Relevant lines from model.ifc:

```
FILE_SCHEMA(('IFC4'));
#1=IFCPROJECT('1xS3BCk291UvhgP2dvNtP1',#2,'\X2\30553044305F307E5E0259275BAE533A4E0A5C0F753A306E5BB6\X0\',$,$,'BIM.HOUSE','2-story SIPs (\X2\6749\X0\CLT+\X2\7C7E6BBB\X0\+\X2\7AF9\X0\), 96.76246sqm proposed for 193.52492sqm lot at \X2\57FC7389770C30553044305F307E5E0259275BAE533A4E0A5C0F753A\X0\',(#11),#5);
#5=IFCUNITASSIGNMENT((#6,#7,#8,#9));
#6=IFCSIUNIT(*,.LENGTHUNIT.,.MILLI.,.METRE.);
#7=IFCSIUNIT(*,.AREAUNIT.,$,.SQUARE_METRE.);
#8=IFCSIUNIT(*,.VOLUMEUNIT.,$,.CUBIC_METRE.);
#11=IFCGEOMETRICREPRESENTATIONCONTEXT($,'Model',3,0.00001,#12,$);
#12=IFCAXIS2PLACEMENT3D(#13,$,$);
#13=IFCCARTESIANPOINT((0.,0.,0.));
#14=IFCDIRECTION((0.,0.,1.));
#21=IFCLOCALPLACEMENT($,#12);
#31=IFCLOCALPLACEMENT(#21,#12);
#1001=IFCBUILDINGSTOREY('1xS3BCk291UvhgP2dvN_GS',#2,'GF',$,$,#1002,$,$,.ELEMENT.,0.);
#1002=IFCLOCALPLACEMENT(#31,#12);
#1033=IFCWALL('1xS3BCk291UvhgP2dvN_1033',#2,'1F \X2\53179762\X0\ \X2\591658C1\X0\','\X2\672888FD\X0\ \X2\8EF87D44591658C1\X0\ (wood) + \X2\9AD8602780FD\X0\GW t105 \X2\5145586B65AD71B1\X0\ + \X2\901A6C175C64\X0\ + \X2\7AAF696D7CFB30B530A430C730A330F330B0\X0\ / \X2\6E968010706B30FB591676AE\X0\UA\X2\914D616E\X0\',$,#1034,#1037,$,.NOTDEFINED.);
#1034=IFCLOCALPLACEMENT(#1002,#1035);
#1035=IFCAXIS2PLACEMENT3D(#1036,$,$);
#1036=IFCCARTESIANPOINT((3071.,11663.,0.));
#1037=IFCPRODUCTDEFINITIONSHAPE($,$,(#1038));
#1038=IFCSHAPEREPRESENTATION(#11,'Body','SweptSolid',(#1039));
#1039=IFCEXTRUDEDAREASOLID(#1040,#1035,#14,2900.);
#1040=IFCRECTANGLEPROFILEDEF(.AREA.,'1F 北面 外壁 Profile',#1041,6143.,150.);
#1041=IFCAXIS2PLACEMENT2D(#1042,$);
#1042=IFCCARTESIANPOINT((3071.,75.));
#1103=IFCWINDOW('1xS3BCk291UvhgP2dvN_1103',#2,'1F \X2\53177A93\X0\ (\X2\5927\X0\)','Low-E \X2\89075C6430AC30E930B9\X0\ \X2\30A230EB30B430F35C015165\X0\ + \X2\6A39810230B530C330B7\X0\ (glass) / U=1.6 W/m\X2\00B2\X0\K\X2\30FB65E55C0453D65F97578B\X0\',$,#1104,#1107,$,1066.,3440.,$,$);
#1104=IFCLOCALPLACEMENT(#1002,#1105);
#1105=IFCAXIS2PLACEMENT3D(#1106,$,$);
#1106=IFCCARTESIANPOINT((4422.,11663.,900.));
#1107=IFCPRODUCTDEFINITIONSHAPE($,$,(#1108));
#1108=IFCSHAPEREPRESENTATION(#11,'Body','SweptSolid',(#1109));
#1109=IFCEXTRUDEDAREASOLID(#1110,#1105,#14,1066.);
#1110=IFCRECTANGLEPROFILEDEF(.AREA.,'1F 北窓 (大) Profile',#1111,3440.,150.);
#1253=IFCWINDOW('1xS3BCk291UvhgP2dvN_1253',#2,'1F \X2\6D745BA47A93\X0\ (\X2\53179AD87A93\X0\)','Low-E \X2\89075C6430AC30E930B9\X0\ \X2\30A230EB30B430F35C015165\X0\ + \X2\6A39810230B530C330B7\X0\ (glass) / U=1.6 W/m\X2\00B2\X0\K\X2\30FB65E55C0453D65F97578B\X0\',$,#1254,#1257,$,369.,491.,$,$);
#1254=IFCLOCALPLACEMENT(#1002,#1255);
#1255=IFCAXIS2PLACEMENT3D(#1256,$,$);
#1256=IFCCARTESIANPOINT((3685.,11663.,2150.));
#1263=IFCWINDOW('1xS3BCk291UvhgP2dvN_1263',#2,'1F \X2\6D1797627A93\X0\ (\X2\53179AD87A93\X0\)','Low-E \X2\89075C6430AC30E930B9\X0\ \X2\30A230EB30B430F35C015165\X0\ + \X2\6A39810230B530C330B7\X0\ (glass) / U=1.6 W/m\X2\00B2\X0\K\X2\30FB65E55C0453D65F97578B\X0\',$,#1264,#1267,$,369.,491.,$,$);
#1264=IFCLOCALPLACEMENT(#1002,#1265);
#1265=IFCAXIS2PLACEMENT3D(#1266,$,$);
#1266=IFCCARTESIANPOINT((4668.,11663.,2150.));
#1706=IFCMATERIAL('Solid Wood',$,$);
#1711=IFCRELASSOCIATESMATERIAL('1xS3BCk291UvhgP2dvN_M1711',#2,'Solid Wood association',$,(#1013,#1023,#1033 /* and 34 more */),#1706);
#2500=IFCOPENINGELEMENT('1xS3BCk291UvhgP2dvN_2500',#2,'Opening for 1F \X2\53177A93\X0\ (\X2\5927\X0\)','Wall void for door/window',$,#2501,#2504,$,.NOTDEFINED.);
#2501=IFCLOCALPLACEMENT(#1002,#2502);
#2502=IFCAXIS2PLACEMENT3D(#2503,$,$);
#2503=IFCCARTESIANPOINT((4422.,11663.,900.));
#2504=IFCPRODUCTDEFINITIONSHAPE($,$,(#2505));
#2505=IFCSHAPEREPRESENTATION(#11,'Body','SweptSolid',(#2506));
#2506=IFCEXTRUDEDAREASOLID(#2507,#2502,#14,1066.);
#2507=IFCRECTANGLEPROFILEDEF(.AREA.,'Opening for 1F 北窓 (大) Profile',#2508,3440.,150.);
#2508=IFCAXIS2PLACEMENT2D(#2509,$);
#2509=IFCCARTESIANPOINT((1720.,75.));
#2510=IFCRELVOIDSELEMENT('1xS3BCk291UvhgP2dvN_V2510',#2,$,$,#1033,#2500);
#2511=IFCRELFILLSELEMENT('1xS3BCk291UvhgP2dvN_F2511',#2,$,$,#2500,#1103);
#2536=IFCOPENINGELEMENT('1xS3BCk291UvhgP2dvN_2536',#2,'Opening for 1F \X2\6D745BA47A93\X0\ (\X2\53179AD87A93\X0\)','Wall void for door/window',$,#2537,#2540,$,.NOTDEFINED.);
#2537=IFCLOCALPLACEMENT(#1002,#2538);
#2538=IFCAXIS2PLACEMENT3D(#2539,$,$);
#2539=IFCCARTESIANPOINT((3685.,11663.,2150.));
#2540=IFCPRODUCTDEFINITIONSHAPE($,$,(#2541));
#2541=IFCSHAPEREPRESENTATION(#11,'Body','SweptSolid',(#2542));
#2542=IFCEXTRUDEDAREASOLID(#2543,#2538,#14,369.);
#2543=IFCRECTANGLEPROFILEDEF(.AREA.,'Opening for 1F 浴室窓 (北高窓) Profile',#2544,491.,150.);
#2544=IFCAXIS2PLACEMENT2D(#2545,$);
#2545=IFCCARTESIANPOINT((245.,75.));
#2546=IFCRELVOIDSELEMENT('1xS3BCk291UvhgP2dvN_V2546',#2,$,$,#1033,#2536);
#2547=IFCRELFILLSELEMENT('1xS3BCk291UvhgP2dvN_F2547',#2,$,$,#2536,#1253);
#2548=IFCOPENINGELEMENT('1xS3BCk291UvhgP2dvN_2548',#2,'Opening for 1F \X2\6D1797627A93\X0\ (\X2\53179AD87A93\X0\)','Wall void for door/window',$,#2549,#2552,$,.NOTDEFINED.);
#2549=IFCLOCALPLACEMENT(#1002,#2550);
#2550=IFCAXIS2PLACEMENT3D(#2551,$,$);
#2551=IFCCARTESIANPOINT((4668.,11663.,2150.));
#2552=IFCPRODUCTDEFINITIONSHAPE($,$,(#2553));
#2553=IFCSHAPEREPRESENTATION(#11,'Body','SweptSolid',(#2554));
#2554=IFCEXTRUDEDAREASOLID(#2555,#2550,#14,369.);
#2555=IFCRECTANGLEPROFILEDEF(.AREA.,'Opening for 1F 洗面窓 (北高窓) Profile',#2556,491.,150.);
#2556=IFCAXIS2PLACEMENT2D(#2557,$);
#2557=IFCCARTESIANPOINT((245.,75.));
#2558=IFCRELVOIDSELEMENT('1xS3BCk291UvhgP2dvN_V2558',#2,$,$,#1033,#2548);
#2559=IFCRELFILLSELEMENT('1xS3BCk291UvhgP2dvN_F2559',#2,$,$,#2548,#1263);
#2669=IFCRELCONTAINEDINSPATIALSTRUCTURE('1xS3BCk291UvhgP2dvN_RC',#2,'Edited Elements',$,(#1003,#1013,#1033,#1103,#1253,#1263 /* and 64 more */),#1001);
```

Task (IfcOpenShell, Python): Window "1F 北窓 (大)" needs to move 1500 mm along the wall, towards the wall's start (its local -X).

```python
import ifcopenshell
import ifcopenshell.api.geometry
import ifcopenshell.util.placement

model = ifcopenshell.open("model.ifc")

window = model.by_guid("1xS3BCk291UvhgP2dvN_1103")
opening = window.FillsVoids[0].RelatingOpeningElement
wall = opening.VoidsElements[0].RelatingBuildingElement

wall_matrix = ifcopenshell.util.placement.get_local_placement(wall.ObjectPlacement)
shift = wall_matrix[:3, 0] * -1500.0
before = ifcopenshell.util.placement.get_local_placement(window.ObjectPlacement)[:3, 3].copy()

# The window is not placed relative to its opening, so move both.
for product in (opening, window):
    matrix = ifcopenshell.util.placement.get_local_placement(product.ObjectPlacement)
    matrix[:3, 3] += shift
    ifcopenshell.api.geometry.edit_object_placement(model, product=product, matrix=matrix, is_si=False)

after = ifcopenshell.util.placement.get_local_placement(window.ObjectPlacement)[:3, 3]
print("window moved by", (after - before).round(3) + 0.0)

model.write("model_v2.ifc")
```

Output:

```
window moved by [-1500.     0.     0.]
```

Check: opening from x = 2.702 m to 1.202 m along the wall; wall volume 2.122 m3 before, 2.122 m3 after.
